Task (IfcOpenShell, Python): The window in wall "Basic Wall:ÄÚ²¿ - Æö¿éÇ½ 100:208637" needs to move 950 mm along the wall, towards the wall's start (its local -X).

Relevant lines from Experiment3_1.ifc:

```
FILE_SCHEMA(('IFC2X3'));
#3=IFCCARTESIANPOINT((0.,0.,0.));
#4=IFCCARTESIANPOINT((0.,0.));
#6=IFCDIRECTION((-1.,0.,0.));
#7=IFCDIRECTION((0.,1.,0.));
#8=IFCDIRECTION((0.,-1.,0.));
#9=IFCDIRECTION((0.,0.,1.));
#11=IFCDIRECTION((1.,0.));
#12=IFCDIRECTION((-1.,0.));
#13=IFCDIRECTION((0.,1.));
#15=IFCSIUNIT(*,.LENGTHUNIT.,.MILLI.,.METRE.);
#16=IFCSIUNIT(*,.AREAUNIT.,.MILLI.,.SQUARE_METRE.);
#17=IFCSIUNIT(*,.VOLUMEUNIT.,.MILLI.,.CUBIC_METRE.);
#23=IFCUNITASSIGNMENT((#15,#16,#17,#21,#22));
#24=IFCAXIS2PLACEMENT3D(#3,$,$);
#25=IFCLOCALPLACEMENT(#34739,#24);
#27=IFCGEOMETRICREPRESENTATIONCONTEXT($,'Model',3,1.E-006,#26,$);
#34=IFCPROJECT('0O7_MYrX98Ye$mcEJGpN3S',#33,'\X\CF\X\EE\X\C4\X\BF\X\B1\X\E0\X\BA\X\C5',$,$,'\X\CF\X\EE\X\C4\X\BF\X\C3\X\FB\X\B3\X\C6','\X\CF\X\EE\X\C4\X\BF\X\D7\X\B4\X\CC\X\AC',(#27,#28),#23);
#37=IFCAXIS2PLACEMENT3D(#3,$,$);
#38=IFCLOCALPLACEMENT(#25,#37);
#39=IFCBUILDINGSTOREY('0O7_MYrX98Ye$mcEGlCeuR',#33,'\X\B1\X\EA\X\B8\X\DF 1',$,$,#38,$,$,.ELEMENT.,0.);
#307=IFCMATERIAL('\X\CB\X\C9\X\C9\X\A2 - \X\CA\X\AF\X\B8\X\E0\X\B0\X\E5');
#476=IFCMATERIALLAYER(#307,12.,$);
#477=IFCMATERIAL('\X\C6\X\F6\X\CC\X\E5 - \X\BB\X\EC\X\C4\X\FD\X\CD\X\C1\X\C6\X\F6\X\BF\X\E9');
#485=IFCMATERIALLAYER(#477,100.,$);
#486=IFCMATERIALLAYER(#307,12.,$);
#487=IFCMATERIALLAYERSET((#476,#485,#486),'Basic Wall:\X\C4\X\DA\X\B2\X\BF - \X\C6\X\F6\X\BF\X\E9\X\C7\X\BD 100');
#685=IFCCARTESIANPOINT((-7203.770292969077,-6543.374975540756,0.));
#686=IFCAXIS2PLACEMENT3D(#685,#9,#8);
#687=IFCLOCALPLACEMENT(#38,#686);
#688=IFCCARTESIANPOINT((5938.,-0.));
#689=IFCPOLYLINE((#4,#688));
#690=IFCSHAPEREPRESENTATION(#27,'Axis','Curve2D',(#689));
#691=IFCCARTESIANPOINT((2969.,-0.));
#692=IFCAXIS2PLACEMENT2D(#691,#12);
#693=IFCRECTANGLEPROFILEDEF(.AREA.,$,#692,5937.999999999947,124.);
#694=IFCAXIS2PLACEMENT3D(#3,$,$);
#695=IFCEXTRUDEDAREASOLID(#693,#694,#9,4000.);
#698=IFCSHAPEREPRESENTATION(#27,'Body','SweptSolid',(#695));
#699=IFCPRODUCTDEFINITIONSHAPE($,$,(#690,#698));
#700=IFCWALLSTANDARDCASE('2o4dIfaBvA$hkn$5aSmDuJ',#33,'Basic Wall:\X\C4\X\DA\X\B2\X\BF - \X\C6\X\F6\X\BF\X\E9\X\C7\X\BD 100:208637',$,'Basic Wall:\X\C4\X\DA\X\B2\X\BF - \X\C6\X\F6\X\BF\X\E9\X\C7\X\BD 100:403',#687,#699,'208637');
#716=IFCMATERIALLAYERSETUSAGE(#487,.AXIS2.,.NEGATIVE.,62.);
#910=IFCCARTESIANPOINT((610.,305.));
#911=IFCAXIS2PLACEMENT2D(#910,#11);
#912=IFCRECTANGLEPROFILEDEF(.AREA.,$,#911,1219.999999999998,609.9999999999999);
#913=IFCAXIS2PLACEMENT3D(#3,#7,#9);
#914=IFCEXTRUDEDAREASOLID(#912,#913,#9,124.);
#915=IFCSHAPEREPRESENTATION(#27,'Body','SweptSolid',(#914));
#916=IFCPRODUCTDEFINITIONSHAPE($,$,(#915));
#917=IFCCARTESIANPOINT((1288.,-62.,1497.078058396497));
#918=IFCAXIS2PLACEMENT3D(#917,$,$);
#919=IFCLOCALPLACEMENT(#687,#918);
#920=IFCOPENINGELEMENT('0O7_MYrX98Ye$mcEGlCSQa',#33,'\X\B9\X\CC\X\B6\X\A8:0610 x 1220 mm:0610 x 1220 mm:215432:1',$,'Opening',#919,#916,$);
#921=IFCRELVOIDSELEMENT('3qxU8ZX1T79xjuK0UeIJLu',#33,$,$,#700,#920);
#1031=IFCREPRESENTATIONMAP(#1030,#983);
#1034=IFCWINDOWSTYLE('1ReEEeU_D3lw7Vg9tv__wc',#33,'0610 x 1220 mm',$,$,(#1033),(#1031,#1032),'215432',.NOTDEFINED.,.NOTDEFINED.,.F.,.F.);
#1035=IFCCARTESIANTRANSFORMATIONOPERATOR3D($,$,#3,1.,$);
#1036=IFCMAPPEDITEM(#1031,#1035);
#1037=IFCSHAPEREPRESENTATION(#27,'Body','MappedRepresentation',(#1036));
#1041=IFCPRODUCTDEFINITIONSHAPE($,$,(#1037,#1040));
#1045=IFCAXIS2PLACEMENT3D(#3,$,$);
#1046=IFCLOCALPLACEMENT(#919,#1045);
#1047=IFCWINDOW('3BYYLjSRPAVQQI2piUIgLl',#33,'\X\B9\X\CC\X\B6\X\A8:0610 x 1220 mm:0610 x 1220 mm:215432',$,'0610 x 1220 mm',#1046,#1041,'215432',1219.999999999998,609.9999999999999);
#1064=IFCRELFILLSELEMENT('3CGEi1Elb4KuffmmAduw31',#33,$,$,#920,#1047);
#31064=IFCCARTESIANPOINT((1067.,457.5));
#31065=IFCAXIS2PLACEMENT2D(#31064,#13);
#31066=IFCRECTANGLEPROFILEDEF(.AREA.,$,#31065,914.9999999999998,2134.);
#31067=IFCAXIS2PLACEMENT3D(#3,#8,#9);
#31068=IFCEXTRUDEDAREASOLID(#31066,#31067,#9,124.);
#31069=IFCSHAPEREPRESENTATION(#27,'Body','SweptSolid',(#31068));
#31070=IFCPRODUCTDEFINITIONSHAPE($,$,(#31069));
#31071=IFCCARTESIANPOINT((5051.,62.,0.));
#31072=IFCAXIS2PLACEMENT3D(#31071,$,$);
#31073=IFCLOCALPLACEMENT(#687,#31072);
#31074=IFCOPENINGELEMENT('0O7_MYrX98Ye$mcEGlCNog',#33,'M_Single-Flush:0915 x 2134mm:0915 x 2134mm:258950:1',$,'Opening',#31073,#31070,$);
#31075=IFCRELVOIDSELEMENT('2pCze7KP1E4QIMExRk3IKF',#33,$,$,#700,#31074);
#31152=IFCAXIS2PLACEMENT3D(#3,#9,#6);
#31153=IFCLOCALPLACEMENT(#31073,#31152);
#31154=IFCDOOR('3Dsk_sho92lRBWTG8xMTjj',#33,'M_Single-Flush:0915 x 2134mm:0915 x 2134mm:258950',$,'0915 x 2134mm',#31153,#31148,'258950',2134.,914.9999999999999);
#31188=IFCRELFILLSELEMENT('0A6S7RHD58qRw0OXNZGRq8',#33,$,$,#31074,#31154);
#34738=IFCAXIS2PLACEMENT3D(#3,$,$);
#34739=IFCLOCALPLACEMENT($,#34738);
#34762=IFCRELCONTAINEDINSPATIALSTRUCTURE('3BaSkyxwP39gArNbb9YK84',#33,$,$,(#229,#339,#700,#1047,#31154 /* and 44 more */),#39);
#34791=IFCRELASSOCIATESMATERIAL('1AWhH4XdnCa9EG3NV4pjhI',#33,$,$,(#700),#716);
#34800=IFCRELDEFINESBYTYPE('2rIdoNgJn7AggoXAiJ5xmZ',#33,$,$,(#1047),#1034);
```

```python
import ifcopenshell
import ifcopenshell.api.geometry
import ifcopenshell.util.placement
import ifcopenshell.util.unit

model = ifcopenshell.open("Experiment3_1.ifc")
unit_scale = ifcopenshell.util.unit.calculate_unit_scale(model)

window = model.by_guid("3BYYLjSRPAVQQI2piUIgLl")
opening = window.FillsVoids[0].RelatingOpeningElement
wall = opening.VoidsElements[0].RelatingBuildingElement

wall_matrix = ifcopenshell.util.placement.get_local_placement(wall.ObjectPlacement)
shift = wall_matrix[:3, 0] * -0.95 / unit_scale
before = ifcopenshell.util.placement.get_local_placement(window.ObjectPlacement)[:3, 3].copy()

# The window is placed relative to its opening, so it follows when the opening moves.
matrix = ifcopenshell.util.placement.get_local_placement(opening.ObjectPlacement)
matrix[:3, 3] += shift
ifcopenshell.api.geometry.edit_object_placement(
    model, product=opening, matrix=matrix, is_si=False, should_transform_children=True
)

after = ifcopenshell.util.placement.get_local_placement(window.ObjectPlacement)[:3, 3]
print("window moved by", (after - before).round(3) + 0.0)

model.write("Experiment3_1_rev.ifc")
```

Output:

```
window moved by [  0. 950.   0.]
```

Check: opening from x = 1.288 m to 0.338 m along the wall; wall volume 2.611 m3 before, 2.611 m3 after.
